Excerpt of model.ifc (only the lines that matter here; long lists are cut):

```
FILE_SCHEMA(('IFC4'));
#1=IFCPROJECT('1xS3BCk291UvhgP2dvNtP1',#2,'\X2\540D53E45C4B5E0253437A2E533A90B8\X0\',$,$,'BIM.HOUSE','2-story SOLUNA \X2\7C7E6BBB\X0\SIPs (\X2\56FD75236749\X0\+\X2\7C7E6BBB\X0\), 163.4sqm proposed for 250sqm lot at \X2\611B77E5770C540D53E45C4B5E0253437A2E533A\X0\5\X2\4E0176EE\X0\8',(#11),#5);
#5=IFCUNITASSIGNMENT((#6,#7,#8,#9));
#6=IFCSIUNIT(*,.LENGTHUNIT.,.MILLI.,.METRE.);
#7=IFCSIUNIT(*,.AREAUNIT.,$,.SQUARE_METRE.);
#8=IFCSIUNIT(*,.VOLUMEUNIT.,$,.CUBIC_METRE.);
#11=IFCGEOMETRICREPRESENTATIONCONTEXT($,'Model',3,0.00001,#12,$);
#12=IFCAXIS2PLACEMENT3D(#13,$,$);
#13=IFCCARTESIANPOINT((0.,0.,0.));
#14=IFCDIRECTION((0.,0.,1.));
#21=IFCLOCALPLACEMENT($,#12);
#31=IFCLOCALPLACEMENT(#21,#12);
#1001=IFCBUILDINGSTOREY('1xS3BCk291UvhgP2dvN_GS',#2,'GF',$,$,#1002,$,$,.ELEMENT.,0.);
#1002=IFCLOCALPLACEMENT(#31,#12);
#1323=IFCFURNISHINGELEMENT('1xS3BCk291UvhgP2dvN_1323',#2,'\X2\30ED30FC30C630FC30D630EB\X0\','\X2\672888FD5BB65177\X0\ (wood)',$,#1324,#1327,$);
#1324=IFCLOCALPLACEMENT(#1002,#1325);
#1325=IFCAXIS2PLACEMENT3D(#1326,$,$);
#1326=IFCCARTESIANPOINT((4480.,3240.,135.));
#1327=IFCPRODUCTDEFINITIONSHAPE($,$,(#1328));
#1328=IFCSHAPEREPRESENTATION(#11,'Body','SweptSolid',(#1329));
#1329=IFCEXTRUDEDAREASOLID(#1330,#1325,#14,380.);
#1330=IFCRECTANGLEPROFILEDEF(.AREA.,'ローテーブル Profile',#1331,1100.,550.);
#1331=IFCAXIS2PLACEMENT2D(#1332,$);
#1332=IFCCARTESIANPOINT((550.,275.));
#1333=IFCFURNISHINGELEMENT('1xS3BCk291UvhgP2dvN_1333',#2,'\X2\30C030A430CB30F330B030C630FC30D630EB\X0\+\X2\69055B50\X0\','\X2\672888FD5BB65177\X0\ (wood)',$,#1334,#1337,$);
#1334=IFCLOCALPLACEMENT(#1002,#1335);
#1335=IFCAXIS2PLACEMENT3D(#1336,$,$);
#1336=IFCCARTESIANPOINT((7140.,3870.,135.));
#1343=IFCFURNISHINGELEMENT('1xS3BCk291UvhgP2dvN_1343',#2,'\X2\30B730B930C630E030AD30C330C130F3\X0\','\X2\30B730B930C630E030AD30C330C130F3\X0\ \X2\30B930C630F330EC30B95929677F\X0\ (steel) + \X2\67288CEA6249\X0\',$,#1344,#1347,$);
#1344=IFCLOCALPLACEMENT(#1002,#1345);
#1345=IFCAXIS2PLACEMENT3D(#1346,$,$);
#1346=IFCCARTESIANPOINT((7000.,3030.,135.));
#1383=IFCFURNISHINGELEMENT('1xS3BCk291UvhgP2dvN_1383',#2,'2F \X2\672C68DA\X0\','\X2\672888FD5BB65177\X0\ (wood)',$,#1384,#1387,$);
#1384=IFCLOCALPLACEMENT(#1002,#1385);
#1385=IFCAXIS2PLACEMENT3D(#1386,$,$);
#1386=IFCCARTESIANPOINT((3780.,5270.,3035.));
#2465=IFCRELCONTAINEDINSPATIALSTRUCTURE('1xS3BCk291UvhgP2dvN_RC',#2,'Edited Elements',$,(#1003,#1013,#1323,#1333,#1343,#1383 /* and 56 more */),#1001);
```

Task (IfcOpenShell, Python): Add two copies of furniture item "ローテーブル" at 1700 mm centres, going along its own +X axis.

```python
import ifcopenshell
import ifcopenshell.api.geometry
import ifcopenshell.api.root
import ifcopenshell.util.element
import ifcopenshell.util.placement
import ifcopenshell.util.unit

model = ifcopenshell.open("model.ifc")
unit_scale = ifcopenshell.util.unit.calculate_unit_scale(model)


def reuse_history(source, copy):
    """copy_class also copies each property set's owner history, people and application; keep the originals."""
    for rel in copy.IsDefinedBy:
        if rel.is_a("IfcRelDefinesByProperties") and (history := rel.RelatingPropertyDefinition.OwnerHistory):
            rel.RelatingPropertyDefinition.OwnerHistory = source.OwnerHistory
            ifcopenshell.util.element.remove_deep2(model, history)


source = model.by_guid("1xS3BCk291UvhgP2dvN_1323")
base = ifcopenshell.util.placement.get_local_placement(source.ObjectPlacement)
step = base[:3, 0] * 1.7 / unit_scale

for i in range(1, 3):
    copy = ifcopenshell.api.root.copy_class(model, product=source)
    copy.Representation = ifcopenshell.util.element.copy_deep(
        model, source.Representation, exclude=["IfcGeometricRepresentationContext", "IfcRepresentationMap"]
    )
    reuse_history(source, copy)
    matrix = base.copy()
    matrix[:3, 3] += i * step
    print("added at", matrix[:3, 3].round(3) + 0.0)
    ifcopenshell.api.geometry.edit_object_placement(model, product=copy, matrix=matrix, is_si=False)

model.write("model_edited.ifc")
```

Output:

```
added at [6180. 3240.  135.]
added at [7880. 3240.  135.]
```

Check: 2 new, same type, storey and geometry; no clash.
